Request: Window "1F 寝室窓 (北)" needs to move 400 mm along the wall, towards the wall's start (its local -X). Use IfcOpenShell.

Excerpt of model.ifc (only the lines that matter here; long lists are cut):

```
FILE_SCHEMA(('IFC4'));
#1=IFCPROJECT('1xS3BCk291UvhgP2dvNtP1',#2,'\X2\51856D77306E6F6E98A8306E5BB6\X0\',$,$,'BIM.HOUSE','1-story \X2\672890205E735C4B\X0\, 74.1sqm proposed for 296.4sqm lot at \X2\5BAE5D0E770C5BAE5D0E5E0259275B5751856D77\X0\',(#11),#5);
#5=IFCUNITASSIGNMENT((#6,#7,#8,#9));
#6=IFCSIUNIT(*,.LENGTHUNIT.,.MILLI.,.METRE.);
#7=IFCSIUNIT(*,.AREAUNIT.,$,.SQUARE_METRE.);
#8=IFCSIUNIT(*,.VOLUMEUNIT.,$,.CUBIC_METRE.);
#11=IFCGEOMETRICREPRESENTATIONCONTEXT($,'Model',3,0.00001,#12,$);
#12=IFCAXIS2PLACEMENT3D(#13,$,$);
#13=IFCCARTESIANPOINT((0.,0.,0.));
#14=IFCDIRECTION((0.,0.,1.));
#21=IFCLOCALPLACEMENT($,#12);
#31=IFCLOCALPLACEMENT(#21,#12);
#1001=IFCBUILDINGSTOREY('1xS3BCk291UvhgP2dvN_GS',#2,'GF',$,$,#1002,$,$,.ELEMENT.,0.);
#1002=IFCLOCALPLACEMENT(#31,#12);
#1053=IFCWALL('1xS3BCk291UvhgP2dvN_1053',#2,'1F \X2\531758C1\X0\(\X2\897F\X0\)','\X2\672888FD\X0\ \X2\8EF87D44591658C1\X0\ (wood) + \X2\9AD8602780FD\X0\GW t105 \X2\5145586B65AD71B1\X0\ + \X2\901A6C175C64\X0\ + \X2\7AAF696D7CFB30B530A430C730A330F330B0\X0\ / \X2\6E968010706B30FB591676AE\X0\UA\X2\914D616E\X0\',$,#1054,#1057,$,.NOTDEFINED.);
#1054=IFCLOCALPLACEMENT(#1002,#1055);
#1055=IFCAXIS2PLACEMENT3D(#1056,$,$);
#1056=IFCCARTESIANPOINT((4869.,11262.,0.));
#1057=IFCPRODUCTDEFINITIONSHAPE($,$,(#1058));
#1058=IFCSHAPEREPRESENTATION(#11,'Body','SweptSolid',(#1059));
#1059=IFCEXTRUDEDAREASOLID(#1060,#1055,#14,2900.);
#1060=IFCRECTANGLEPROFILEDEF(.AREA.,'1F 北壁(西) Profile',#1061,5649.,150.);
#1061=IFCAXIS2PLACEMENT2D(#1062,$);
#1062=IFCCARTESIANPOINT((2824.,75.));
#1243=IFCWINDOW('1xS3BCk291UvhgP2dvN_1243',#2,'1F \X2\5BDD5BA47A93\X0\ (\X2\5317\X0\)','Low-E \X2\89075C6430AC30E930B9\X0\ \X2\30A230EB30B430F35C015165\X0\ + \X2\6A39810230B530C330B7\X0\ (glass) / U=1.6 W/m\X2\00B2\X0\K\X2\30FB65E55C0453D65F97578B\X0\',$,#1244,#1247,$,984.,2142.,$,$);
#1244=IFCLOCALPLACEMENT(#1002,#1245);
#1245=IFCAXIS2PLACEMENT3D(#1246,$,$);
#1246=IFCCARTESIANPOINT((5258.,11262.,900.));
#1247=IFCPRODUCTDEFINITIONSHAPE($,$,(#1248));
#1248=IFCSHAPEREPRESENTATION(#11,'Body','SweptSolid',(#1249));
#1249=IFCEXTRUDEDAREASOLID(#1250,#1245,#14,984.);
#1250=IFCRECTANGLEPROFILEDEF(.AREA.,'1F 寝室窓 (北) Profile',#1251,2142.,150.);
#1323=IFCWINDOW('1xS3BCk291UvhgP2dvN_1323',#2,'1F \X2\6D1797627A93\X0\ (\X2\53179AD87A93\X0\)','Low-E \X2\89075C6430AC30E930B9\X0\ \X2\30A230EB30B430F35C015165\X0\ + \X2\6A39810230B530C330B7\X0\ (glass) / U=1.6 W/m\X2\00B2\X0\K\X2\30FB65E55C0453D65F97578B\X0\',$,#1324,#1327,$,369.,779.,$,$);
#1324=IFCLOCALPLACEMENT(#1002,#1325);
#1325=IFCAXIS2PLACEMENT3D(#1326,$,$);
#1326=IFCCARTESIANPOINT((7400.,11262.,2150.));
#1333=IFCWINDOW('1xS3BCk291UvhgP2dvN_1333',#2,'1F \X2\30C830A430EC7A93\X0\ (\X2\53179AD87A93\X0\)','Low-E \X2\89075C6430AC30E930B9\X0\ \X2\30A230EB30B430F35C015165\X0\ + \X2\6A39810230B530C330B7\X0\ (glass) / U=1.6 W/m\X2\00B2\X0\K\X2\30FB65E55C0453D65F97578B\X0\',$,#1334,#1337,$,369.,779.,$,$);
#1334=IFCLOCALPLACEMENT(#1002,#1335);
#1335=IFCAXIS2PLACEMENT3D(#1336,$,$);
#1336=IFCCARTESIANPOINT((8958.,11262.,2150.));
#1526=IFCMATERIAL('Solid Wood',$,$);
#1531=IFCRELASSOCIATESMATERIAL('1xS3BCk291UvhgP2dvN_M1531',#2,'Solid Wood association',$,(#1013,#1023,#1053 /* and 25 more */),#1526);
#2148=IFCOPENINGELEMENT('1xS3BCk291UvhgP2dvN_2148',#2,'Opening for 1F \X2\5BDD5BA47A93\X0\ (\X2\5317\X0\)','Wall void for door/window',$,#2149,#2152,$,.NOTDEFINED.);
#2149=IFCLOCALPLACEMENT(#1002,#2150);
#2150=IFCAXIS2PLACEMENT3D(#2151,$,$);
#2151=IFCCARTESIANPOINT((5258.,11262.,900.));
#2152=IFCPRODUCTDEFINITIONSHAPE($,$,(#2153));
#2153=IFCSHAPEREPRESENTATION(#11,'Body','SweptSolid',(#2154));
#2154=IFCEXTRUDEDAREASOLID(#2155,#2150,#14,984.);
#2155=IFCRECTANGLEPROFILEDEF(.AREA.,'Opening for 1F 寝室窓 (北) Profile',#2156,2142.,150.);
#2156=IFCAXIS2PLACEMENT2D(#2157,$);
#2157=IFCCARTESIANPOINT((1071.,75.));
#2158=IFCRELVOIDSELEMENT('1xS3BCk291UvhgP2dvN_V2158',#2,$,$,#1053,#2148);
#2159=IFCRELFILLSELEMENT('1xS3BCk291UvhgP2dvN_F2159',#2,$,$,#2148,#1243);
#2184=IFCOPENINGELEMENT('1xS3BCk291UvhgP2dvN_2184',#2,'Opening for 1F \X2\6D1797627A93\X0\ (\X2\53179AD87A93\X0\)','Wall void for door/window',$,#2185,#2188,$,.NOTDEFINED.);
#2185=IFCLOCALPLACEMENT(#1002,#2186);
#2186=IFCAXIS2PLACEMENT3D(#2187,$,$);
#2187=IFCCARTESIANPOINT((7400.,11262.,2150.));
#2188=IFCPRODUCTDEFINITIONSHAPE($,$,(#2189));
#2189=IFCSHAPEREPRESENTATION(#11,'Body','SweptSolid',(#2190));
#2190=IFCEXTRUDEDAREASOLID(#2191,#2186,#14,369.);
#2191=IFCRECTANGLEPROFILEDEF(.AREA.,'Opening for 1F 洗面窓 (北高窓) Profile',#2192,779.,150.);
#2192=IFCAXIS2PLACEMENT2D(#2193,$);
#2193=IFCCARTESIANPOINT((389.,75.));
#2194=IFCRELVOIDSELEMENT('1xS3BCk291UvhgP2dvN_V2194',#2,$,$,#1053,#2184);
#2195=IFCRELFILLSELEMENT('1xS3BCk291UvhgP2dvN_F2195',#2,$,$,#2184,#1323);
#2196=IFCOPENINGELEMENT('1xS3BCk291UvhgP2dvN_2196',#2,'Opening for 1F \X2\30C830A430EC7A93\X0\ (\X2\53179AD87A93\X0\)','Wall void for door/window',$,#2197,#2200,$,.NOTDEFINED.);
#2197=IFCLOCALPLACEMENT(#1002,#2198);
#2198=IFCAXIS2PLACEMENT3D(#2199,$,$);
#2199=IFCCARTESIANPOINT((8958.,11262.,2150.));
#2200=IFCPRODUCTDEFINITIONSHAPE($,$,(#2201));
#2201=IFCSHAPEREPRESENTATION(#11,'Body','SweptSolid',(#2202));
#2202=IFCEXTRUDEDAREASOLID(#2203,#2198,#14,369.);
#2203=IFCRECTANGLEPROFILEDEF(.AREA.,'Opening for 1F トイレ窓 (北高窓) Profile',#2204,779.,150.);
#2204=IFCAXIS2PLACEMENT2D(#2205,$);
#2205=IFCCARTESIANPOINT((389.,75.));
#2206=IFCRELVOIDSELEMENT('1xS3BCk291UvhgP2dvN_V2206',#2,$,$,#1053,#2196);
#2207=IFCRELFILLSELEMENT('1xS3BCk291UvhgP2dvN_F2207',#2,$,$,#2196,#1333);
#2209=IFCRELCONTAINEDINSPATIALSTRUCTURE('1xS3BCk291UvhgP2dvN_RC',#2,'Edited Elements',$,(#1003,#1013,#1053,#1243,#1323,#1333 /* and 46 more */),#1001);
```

```python
import ifcopenshell
import ifcopenshell.api.geometry
import ifcopenshell.util.placement

model = ifcopenshell.open("model.ifc")

window = model.by_guid("1xS3BCk291UvhgP2dvN_1243")
opening = window.FillsVoids[0].RelatingOpeningElement
wall = opening.VoidsElements[0].RelatingBuildingElement

wall_matrix = ifcopenshell.util.placement.get_local_placement(wall.ObjectPlacement)
shift = wall_matrix[:3, 0] * -400.0
before = ifcopenshell.util.placement.get_local_placement(window.ObjectPlacement)[:3, 3].copy()

# The window is not placed relative to its opening, so move both.
for product in (opening, window):
    matrix = ifcopenshell.util.placement.get_local_placement(product.ObjectPlacement)
    matrix[:3, 3] += shift
    ifcopenshell.api.geometry.edit_object_placement(model, product=product, matrix=matrix, is_si=False)

after = ifcopenshell.util.placement.get_local_placement(window.ObjectPlacement)[:3, 3]
print("window moved by", (after - before).round(3) + 0.0)

model.write("model_v2.ifc")
```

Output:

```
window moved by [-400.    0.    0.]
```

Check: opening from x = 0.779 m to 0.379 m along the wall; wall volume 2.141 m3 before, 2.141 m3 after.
